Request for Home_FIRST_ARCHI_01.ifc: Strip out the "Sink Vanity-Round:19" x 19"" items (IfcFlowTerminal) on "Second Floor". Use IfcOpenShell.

First a look at what the model holds.

```python
import ifcopenshell
import ifcopenshell.util.element

model = ifcopenshell.open("Home_FIRST_ARCHI_01.ifc")
print(model.schema)
storey = next(s for s in model.by_type("IfcBuildingStorey") if s.Name == "Second Floor")
terminals = [e for e in ifcopenshell.util.element.get_decomposition(storey) if e.is_a("IfcFlowTerminal")]
seen = {}
for e in terminals:
    element_type = ifcopenshell.util.element.get_type(e)
    name = element_type.Name if element_type not in (None, e) else None
    seen[name] = seen.get(name, 0) + 1
for name, count in sorted(seen.items(), key=str):
    print(count, "x", name)
```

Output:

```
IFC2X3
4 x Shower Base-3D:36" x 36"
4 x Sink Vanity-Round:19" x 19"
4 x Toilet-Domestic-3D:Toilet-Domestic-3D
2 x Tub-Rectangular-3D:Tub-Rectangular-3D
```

```python
import ifcopenshell
import ifcopenshell.api.root
import ifcopenshell.util.element

model = ifcopenshell.open("Home_FIRST_ARCHI_01.ifc")

storey = next(s for s in model.by_type("IfcBuildingStorey") if s.Name == "Second Floor")
terminals = [e for e in ifcopenshell.util.element.get_decomposition(storey) if e.is_a("IfcFlowTerminal")]
targets = [e for e in terminals if (t := ifcopenshell.util.element.get_type(e)) not in (None, e) and t.Name == 'Sink Vanity-Round:19" x 19"']

for e in targets:
    ifcopenshell.api.root.remove_product(model, product=e)
print(len(targets), "removed")

model.write("Home_FIRST_ARCHI_01_rev.ifc")
```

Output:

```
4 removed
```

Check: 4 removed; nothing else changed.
